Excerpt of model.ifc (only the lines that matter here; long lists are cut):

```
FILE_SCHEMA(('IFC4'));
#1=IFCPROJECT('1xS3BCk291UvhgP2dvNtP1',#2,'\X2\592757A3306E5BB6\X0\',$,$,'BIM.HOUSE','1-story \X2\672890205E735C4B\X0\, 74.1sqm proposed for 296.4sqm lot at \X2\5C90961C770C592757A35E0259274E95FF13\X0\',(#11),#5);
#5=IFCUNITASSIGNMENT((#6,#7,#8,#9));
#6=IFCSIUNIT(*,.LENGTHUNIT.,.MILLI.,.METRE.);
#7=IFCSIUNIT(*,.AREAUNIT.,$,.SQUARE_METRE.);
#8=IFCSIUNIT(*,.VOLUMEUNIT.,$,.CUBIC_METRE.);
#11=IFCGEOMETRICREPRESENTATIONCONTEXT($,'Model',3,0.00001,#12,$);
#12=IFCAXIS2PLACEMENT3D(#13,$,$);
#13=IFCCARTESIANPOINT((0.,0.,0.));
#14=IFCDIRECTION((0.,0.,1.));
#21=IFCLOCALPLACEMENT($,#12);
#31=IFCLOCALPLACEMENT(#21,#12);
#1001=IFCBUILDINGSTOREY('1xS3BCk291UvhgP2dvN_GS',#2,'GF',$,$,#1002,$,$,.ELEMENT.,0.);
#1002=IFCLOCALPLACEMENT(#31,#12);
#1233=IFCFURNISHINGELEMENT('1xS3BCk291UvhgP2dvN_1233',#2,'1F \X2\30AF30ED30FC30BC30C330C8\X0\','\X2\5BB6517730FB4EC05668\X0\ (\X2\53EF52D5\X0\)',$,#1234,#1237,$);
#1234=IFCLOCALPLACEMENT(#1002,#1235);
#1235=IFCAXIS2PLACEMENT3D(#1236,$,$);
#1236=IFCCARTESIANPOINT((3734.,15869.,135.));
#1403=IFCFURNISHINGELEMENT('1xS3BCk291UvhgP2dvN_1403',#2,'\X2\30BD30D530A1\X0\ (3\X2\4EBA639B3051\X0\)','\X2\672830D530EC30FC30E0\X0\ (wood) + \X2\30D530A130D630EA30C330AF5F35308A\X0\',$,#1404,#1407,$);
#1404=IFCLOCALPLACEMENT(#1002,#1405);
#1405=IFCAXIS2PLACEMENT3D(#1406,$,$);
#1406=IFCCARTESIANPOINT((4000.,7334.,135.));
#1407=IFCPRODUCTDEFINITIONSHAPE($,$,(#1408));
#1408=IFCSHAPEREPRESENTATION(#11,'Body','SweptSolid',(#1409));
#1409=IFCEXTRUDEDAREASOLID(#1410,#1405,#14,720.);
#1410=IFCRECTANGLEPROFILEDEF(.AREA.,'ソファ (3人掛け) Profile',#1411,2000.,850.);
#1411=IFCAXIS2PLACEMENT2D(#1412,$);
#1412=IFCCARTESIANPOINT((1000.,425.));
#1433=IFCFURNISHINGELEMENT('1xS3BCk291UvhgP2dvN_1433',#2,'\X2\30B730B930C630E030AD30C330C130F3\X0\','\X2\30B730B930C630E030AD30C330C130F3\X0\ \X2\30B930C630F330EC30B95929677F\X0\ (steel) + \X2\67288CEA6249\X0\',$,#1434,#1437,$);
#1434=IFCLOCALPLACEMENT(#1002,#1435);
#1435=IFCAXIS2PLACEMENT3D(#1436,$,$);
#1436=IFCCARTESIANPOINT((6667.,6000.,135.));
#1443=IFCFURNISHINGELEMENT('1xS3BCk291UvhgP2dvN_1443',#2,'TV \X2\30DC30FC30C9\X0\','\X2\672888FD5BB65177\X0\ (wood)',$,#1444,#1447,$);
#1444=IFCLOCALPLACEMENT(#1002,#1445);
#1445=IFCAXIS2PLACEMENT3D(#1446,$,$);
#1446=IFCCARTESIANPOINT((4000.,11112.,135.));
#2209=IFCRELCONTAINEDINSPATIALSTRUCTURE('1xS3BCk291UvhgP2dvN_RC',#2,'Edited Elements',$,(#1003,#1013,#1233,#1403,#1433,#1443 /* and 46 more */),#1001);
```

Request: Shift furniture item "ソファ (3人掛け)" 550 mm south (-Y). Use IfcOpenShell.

```python
import ifcopenshell
import ifcopenshell.api.geometry
import ifcopenshell.util.placement
import ifcopenshell.util.unit

model = ifcopenshell.open("model.ifc")
unit_scale = ifcopenshell.util.unit.calculate_unit_scale(model)

item = model.by_id(1403)
matrix = ifcopenshell.util.placement.get_local_placement(item.ObjectPlacement)
matrix[1, 3] -= 0.55 / unit_scale
ifcopenshell.api.geometry.edit_object_placement(model, product=item, matrix=matrix, is_si=False)

print(ifcopenshell.util.placement.get_local_placement(item.ObjectPlacement).round(3) + 0.0)

model.write("model_edited.ifc")
```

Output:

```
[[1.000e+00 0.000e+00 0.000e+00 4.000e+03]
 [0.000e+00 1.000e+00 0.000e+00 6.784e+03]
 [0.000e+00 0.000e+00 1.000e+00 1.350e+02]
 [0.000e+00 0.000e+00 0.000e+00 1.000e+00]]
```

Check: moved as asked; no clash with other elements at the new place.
